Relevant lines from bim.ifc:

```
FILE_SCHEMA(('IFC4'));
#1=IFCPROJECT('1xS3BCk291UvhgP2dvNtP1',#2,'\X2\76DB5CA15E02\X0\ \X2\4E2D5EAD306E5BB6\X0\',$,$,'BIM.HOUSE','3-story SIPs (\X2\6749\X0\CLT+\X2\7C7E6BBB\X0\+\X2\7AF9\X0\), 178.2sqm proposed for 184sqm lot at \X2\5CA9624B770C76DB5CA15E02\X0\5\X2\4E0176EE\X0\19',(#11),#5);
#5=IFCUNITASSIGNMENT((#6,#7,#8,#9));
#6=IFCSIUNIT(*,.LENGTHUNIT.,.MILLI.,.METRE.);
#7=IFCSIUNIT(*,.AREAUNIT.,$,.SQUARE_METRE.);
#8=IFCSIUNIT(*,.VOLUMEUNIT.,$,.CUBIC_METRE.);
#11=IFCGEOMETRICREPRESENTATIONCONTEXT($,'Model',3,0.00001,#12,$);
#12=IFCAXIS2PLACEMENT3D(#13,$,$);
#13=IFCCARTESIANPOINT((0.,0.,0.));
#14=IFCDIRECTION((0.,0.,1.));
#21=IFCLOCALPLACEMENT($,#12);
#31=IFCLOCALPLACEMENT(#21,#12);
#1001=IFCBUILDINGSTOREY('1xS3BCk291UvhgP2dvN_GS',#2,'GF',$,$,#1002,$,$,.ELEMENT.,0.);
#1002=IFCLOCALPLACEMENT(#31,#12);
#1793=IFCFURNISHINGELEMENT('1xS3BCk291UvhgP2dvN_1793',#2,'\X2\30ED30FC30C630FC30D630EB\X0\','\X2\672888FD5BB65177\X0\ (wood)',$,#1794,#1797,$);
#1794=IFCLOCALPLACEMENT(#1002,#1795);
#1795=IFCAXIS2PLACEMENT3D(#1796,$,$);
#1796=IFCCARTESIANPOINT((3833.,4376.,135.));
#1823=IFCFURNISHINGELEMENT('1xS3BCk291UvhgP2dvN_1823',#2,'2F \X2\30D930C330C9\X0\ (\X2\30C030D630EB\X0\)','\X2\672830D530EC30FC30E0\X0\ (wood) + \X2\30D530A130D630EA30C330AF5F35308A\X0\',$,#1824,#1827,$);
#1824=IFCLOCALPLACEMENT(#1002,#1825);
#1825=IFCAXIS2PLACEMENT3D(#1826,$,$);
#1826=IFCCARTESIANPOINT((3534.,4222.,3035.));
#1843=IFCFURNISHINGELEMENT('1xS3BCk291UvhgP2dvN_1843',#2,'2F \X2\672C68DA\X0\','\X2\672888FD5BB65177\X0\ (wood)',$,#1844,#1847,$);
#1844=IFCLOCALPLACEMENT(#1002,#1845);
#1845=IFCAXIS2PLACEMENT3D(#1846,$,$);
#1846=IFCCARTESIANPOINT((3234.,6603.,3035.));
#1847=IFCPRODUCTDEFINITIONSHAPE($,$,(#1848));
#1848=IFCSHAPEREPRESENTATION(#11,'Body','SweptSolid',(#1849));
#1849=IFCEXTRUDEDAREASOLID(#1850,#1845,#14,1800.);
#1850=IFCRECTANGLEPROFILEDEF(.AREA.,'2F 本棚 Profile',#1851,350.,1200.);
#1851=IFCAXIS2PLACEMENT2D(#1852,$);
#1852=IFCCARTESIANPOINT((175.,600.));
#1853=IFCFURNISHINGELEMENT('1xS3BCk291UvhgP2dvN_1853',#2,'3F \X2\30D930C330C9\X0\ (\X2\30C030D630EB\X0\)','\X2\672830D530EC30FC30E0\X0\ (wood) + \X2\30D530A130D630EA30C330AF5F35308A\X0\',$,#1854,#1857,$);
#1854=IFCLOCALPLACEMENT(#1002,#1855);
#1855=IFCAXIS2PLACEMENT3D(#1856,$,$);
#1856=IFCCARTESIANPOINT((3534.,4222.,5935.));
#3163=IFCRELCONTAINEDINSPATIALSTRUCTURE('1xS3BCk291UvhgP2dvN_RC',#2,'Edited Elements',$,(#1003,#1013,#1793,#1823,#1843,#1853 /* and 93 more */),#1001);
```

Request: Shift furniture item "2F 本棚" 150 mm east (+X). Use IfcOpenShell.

```python
import ifcopenshell
import ifcopenshell.api.geometry
import ifcopenshell.util.placement

model = ifcopenshell.open("bim.ifc")

item = model.by_id(1843)
matrix = ifcopenshell.util.placement.get_local_placement(item.ObjectPlacement)
matrix[0, 3] += 150.0
ifcopenshell.api.geometry.edit_object_placement(model, product=item, matrix=matrix, is_si=False)

print(ifcopenshell.util.placement.get_local_placement(item.ObjectPlacement).round(3) + 0.0)

model.write("bim_rev.ifc")
```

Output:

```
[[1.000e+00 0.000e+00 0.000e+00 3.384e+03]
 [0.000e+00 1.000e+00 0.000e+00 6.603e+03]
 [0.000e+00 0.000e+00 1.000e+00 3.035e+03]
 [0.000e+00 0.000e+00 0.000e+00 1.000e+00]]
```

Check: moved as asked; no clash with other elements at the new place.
